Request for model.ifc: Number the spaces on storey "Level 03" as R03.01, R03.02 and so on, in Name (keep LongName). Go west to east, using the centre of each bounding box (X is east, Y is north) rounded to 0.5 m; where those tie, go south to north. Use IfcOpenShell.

First a look at what the model holds.

```python
import ifcopenshell
import ifcopenshell.util.element
import ifcopenshell.util.placement

model = ifcopenshell.open("model.ifc")
print(model.schema)
storey = next(s for s in model.by_type("IfcBuildingStorey") if s.Name == "Level 03")
spaces = [e for e in ifcopenshell.util.element.get_decomposition(storey) if e.is_a("IfcSpace")]
for e in sorted(spaces, key=lambda e: e.id()):
    origin = ifcopenshell.util.placement.get_local_placement(e.ObjectPlacement)[:3, 3]
    print(e.id(), e.Name, e.LongName, origin.round(2) + 0.0, sep=" | ")
```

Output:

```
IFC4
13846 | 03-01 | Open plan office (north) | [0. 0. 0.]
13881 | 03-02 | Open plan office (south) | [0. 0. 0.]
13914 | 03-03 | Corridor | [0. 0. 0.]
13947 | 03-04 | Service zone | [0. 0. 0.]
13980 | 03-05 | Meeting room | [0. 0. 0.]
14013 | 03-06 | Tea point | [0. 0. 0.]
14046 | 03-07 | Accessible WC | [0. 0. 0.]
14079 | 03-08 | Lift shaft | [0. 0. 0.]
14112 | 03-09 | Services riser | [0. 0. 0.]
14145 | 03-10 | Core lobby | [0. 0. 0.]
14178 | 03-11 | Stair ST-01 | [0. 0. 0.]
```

```python
import ifcopenshell
import ifcopenshell.geom
import ifcopenshell.util.element
import ifcopenshell.util.shape

model = ifcopenshell.open("model.ifc")
settings = ifcopenshell.geom.settings()
settings.set("use-world-coords", True)


def centre(element):
    shape = ifcopenshell.geom.create_shape(settings, element)
    return ifcopenshell.util.shape.get_bbox_centroid(shape.geometry)


storey = next(s for s in model.by_type("IfcBuildingStorey") if s.Name == "Level 03")
spaces = [e for e in ifcopenshell.util.element.get_decomposition(storey) if e.is_a("IfcSpace")]

# Insertion points can sit at a corner or the storey origin, so sort by the geometry (in metres).
centres = {e: centre(e) for e in spaces}
spaces.sort(key=lambda e: (round(centres[e][0] / 0.5), centres[e][1]))

for i, e in enumerate(spaces, start=1):
    number = f"R03.{i:02d}"
    e.Name = number
    print(e.id(), number)

model.write("model-out.ifc")
```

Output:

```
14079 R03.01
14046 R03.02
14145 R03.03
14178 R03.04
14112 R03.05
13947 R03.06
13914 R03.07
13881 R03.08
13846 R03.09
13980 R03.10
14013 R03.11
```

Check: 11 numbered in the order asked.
